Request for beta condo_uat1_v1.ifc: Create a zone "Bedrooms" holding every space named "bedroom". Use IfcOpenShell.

First a look at what the model holds.

```python
import ifcopenshell

model = ifcopenshell.open("beta condo_uat1_v1.ifc")
print(model.schema)
seen = {}
for space in model.by_type("IfcSpace"):
    seen[space.LongName] = seen.get(space.LongName, 0) + 1
for name, count in sorted(seen.items(), key=str):
    print(count, "x", name)
print("zones:", [z.Name for z in model.by_type("IfcZone")][:20])
```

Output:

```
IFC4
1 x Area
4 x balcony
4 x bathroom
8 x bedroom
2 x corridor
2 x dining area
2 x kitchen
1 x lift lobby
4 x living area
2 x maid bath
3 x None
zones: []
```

```python
import ifcopenshell
import ifcopenshell.api.group
import ifcopenshell.api.root

model = ifcopenshell.open("beta condo_uat1_v1.ifc")

names = {"bedroom"}
spaces = [s for s in model.by_type("IfcSpace") if s.LongName in names]

zone = ifcopenshell.api.root.create_entity(model, ifc_class="IfcZone", name="Bedrooms")
ifcopenshell.api.group.assign_group(model, products=spaces, group=zone)
print(len(spaces), "spaces in", zone.Name)

model.write("beta condo_uat1_v1-out.ifc")
```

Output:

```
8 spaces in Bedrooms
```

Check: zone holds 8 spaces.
